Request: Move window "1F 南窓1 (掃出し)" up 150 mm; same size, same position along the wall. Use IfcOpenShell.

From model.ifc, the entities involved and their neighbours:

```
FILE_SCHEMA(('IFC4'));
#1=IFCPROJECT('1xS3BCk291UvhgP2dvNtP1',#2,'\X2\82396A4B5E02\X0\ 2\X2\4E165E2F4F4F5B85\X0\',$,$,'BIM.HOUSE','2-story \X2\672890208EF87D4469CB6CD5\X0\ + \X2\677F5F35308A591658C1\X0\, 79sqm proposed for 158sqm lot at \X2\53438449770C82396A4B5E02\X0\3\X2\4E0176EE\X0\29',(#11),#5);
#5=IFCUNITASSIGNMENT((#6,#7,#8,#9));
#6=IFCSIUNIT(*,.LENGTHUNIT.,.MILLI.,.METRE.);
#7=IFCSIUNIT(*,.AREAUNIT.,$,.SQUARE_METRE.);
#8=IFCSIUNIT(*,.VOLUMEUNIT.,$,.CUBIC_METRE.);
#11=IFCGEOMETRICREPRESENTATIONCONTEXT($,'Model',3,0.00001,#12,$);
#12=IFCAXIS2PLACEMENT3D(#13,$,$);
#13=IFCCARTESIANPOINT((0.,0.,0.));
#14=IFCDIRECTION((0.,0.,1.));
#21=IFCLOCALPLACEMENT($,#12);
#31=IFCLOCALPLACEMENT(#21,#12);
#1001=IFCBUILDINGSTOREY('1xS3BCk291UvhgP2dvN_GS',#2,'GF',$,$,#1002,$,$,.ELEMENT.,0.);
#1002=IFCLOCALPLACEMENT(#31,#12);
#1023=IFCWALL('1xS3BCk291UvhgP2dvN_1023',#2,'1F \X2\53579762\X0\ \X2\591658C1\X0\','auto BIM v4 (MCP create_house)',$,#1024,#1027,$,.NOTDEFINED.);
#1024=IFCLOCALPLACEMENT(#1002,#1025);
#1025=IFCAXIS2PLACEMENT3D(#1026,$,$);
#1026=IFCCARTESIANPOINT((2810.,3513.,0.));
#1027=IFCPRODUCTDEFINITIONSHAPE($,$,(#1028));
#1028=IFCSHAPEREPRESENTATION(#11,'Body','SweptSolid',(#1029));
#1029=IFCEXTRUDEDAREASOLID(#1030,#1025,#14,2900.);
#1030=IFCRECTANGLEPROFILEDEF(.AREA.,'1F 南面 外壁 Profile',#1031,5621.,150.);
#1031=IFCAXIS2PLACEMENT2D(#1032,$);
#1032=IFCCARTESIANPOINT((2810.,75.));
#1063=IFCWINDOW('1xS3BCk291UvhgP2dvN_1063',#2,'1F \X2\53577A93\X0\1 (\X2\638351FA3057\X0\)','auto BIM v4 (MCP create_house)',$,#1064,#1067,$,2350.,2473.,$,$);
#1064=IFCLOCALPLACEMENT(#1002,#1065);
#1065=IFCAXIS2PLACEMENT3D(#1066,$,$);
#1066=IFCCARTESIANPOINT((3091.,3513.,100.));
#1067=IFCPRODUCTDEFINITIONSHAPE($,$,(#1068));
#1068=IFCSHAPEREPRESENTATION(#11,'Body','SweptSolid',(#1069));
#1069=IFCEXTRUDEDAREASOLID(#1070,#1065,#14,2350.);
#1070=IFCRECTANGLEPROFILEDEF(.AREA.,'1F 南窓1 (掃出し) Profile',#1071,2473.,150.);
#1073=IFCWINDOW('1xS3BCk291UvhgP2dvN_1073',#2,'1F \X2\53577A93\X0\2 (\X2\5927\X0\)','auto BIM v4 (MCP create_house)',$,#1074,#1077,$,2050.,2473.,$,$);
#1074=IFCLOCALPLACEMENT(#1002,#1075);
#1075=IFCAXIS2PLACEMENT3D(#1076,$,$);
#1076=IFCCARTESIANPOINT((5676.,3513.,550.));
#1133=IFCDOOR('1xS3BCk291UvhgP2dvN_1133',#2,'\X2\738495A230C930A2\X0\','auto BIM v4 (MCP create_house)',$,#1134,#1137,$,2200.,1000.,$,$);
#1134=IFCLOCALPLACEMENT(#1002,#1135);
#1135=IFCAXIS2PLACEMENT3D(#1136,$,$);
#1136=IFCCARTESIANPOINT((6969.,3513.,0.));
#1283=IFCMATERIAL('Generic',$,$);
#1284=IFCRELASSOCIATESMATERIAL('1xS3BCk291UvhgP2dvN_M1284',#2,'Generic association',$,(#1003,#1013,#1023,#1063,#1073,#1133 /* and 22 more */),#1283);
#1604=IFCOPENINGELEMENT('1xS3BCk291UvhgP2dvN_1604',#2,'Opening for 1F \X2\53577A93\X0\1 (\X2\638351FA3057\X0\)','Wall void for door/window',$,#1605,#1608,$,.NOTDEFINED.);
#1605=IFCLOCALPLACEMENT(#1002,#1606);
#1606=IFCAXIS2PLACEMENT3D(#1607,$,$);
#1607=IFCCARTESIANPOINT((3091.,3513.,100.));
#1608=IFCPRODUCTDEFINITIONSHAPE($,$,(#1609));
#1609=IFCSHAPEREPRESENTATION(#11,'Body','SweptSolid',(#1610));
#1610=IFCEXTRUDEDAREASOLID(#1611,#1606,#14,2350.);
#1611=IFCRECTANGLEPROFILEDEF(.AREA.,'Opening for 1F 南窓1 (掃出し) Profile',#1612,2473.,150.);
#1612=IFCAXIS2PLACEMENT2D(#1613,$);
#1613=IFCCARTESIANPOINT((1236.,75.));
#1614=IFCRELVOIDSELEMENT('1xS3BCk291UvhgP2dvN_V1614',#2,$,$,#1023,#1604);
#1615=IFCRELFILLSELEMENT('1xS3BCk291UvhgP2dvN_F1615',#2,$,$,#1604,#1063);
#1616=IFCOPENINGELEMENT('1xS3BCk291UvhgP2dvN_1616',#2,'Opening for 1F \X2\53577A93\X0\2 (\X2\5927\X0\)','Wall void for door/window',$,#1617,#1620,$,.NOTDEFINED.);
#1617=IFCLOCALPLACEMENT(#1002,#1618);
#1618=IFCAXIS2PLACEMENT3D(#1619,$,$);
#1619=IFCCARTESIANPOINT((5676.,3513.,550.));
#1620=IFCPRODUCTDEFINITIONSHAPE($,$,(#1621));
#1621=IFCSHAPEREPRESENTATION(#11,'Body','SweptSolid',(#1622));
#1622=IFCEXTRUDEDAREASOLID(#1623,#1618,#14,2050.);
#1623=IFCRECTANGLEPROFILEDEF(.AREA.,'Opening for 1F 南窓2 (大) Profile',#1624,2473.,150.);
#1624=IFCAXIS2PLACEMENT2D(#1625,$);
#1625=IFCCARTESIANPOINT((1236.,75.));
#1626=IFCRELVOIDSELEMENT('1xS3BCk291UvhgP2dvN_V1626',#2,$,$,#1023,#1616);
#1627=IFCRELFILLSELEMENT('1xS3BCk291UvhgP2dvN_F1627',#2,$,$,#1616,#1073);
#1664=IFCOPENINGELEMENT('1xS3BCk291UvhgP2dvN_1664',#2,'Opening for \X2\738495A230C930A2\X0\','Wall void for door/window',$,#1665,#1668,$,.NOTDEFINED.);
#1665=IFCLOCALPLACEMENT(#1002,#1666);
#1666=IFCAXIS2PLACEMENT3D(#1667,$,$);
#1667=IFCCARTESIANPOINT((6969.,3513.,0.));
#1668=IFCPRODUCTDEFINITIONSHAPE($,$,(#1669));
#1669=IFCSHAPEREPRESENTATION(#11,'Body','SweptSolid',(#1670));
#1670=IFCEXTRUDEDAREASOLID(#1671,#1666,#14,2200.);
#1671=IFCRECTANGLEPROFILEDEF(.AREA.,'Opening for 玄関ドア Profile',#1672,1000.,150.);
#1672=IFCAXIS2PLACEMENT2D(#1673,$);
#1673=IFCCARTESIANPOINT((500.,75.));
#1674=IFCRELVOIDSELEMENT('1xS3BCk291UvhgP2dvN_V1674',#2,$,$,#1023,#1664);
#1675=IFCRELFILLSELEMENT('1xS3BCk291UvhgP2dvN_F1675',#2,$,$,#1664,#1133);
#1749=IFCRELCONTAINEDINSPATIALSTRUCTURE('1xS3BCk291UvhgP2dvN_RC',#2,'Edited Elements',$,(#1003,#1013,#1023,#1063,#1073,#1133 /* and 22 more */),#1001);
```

```python
import numpy as np
import ifcopenshell
import ifcopenshell.api.geometry
import ifcopenshell.util.placement
import ifcopenshell.util.unit

model = ifcopenshell.open("model.ifc")
unit_scale = ifcopenshell.util.unit.calculate_unit_scale(model)

window = model.by_guid("1xS3BCk291UvhgP2dvN_1063")
opening = window.FillsVoids[0].RelatingOpeningElement
dz = 150.0

shift = np.array([0.0, 0.0, dz])
# The window is not placed relative to its opening, so move both.
for product in (opening, window):
    matrix = ifcopenshell.util.placement.get_local_placement(product.ObjectPlacement)
    matrix[:3, 3] += shift
    ifcopenshell.api.geometry.edit_object_placement(model, product=product, matrix=matrix, is_si=False)

print(f"moved by {dz * unit_scale:+.3f} m")

model.write("model_updated.ifc")
```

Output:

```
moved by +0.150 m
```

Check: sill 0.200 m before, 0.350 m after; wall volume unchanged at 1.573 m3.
